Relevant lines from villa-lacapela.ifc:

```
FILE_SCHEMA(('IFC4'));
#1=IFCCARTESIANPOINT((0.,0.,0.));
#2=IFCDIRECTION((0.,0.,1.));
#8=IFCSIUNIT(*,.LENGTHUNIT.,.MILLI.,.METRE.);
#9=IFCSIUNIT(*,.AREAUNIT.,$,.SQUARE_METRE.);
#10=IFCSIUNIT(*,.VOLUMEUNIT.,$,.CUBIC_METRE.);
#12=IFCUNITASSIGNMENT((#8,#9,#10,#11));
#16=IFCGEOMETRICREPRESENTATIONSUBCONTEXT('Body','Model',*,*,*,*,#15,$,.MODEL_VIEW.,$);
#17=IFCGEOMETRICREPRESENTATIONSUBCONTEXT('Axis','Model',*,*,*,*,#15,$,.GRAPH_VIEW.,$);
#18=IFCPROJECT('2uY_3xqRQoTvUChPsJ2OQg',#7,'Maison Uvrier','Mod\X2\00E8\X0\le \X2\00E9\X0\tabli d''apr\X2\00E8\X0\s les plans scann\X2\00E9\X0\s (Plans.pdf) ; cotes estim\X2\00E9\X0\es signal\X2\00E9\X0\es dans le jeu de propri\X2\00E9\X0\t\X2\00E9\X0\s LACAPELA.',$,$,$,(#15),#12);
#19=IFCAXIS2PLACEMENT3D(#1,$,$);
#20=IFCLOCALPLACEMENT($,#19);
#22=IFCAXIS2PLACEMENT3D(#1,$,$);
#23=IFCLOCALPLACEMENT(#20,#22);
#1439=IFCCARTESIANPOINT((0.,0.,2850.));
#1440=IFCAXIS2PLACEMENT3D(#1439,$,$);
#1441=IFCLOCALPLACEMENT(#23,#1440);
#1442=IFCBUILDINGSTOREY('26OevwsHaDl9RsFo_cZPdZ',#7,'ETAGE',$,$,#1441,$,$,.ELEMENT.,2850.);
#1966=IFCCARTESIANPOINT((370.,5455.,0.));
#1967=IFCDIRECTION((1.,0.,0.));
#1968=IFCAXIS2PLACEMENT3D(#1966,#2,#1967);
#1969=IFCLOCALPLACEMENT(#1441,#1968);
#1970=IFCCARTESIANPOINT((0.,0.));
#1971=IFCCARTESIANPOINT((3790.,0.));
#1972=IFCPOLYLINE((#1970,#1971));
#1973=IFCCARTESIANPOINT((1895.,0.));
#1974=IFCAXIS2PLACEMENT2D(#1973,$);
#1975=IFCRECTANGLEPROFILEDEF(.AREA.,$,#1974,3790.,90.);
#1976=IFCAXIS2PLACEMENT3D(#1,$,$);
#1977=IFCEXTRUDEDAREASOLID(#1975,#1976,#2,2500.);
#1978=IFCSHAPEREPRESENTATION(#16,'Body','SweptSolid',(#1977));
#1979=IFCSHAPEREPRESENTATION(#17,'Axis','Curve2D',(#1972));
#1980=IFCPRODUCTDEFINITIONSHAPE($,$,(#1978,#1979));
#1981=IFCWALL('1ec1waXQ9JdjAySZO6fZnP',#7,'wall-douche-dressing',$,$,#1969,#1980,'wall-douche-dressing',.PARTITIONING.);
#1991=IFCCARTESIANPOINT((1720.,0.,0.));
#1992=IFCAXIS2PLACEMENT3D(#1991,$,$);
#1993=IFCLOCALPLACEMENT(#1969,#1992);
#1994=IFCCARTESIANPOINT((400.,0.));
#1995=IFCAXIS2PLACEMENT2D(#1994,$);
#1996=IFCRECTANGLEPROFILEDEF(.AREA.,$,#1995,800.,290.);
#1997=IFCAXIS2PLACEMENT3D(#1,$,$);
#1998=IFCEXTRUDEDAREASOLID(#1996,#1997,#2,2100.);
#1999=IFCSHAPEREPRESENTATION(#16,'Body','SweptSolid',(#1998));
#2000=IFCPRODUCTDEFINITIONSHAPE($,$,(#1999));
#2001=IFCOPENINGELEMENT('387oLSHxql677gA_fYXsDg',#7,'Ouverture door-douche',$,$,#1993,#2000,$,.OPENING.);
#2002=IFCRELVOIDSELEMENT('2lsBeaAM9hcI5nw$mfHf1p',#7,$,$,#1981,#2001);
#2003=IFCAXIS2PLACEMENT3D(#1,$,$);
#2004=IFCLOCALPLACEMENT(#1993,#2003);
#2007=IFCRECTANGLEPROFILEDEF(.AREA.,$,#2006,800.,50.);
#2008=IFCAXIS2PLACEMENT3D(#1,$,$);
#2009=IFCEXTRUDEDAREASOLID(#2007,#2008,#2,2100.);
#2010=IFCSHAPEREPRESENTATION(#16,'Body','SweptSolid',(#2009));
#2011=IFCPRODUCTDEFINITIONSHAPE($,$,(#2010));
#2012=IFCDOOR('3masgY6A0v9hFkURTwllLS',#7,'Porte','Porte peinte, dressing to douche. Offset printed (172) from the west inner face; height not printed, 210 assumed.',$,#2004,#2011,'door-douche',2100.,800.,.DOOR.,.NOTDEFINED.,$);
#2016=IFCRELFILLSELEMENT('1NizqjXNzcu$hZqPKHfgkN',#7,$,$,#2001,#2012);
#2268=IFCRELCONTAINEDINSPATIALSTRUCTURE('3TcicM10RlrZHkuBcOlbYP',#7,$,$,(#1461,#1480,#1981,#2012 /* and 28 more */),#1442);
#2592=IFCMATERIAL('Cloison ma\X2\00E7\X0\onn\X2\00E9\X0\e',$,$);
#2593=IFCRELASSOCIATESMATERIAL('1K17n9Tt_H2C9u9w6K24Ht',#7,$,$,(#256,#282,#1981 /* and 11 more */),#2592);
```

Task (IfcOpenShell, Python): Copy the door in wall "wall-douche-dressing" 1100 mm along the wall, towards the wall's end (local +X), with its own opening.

```python
import ifcopenshell
import ifcopenshell.api.feature
import ifcopenshell.api.geometry
import ifcopenshell.api.root
import ifcopenshell.geom
import ifcopenshell.util.element
import ifcopenshell.util.placement
import ifcopenshell.util.shape
import ifcopenshell.util.unit

model = ifcopenshell.open("villa-lacapela.ifc")
unit_scale = ifcopenshell.util.unit.calculate_unit_scale(model)
settings = ifcopenshell.geom.settings()


def volume(element):
    """Net volume in cubic metres, openings subtracted."""
    shape = ifcopenshell.geom.create_shape(settings, element)
    return ifcopenshell.util.shape.get_volume(shape.geometry)


def reuse_history(source, copy):
    """copy_class also copies each property set's owner history, people and application; keep the originals."""
    for rel in copy.IsDefinedBy:
        if rel.is_a("IfcRelDefinesByProperties") and (history := rel.RelatingPropertyDefinition.OwnerHistory):
            rel.RelatingPropertyDefinition.OwnerHistory = source.OwnerHistory
            ifcopenshell.util.element.remove_deep2(model, history)


door = model.by_guid("3masgY6A0v9hFkURTwllLS")
opening = door.FillsVoids[0].RelatingOpeningElement
wall = opening.VoidsElements[0].RelatingBuildingElement
before = volume(wall)
shift = ifcopenshell.util.placement.get_local_placement(wall.ObjectPlacement)[:3, 0] * 1.1 / unit_scale

# copy_class copies the void relationship, type, container and properties, but no geometry.
new_opening = ifcopenshell.api.root.copy_class(model, product=opening)
new_opening.Representation = ifcopenshell.util.element.copy_deep(
    model, opening.Representation, exclude=["IfcGeometricRepresentationContext", "IfcRepresentationMap"]
)
new_door = ifcopenshell.api.root.copy_class(model, product=door)
new_door.Representation = ifcopenshell.util.element.copy_deep(
    model, door.Representation, exclude=["IfcGeometricRepresentationContext", "IfcRepresentationMap"]
)
new_door.Tag = None
reuse_history(door, new_door)
ifcopenshell.api.feature.add_filling(model, opening=new_opening, element=new_door)

for old, new in ((opening, new_opening), (door, new_door)):
    matrix = ifcopenshell.util.placement.get_local_placement(old.ObjectPlacement)
    matrix[:3, 3] += shift
    ifcopenshell.api.geometry.edit_object_placement(model, product=new, matrix=matrix, is_si=False)

after = volume(wall)

print(f"wall volume {before:.3f} -> {after:.3f} m3")

model.write("villa-lacapela_updated.ifc")
```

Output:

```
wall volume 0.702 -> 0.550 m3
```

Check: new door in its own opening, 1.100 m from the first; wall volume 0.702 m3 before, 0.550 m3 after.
